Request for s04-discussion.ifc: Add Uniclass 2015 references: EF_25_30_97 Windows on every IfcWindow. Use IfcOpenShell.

First a look at what the model holds.

```python
import ifcopenshell

model = ifcopenshell.open("s04-discussion.ifc")
print(model.schema)
print("classifications:", [c.Name for c in model.by_type("IfcClassification")])
for ifc_class in ("IfcDoor", "IfcRoof", "IfcStair", "IfcWall", "IfcWindow"):
    print(ifc_class, len(model.by_type(ifc_class)))
```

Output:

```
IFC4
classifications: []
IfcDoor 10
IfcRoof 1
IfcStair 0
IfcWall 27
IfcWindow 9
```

```python
import ifcopenshell
import ifcopenshell.api.classification

model = ifcopenshell.open("s04-discussion.ifc")

system = ifcopenshell.api.classification.add_classification(model, classification="Uniclass 2015")

codes = {
    "IfcWindow": ("EF_25_30_97", "Windows"),
}
for ifc_class, (code, name) in codes.items():
    products = model.by_type(ifc_class)
    ifcopenshell.api.classification.add_reference(
        model, products=products, classification=system, identification=code, name=name
    )
    print(code, len(products))

model.write("s04-discussion_updated.ifc")
```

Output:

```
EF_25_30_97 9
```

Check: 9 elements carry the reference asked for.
